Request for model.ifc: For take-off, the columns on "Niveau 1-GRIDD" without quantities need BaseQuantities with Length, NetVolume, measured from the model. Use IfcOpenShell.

First a look at what the model holds.

```python
import ifcopenshell
import ifcopenshell.util.element
import ifcopenshell.util.unit

model = ifcopenshell.open("model.ifc")
print(model.schema)
for unit_type in ("LENGTHUNIT", "AREAUNIT", "VOLUMEUNIT"):
    print(unit_type, ifcopenshell.util.unit.calculate_unit_scale(model, unit_type))
storey = next(s for s in model.by_type("IfcBuildingStorey") if s.Name == "Niveau 1-GRIDD")
columns = [e for e in ifcopenshell.util.element.get_decomposition(storey) if e.is_a("IfcColumn")]
for e in sorted(columns, key=lambda e: e.id()):
    print(e.id(), e.is_a(), e.Name, list(ifcopenshell.util.element.get_psets(e, qtos_only=True)), sep=" | ")
```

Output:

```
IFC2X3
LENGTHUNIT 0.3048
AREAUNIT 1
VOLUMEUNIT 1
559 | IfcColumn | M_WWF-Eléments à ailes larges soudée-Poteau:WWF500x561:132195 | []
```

```python
import ifcopenshell
import ifcopenshell.api.pset
import ifcopenshell.geom
import ifcopenshell.util.element
import ifcopenshell.util.shape
import ifcopenshell.util.unit

model = ifcopenshell.open("model.ifc")
unit_scale = ifcopenshell.util.unit.calculate_unit_scale(model)
volume_scale = ifcopenshell.util.unit.calculate_unit_scale(model, "VOLUMEUNIT")
settings = ifcopenshell.geom.settings()

storey = next(s for s in model.by_type("IfcBuildingStorey") if s.Name == "Niveau 1-GRIDD")
columns = [e for e in ifcopenshell.util.element.get_decomposition(storey) if e.is_a("IfcColumn")]

for e in sorted(columns, key=lambda e: e.id()):
    if ifcopenshell.util.element.get_psets(e, qtos_only=True, should_inherit=False):
        continue
    # Geometry comes back in metres, in the element's own axes.
    shape = ifcopenshell.geom.create_shape(settings, e)
    values = {
        "Length": ifcopenshell.util.shape.get_z(shape.geometry) / unit_scale,
        "NetVolume": ifcopenshell.util.shape.get_volume(shape.geometry) / volume_scale,
    }
    qto = ifcopenshell.api.pset.add_qto(model, product=e, name="BaseQuantities")
    ifcopenshell.api.pset.edit_qto(model, qto=qto, properties=values)
    print(e.id(), {k: round(v, 3) for k, v in values.items()})

model.write("model_v2.ifc")
```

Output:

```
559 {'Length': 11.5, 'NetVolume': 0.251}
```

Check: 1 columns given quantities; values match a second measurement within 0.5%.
